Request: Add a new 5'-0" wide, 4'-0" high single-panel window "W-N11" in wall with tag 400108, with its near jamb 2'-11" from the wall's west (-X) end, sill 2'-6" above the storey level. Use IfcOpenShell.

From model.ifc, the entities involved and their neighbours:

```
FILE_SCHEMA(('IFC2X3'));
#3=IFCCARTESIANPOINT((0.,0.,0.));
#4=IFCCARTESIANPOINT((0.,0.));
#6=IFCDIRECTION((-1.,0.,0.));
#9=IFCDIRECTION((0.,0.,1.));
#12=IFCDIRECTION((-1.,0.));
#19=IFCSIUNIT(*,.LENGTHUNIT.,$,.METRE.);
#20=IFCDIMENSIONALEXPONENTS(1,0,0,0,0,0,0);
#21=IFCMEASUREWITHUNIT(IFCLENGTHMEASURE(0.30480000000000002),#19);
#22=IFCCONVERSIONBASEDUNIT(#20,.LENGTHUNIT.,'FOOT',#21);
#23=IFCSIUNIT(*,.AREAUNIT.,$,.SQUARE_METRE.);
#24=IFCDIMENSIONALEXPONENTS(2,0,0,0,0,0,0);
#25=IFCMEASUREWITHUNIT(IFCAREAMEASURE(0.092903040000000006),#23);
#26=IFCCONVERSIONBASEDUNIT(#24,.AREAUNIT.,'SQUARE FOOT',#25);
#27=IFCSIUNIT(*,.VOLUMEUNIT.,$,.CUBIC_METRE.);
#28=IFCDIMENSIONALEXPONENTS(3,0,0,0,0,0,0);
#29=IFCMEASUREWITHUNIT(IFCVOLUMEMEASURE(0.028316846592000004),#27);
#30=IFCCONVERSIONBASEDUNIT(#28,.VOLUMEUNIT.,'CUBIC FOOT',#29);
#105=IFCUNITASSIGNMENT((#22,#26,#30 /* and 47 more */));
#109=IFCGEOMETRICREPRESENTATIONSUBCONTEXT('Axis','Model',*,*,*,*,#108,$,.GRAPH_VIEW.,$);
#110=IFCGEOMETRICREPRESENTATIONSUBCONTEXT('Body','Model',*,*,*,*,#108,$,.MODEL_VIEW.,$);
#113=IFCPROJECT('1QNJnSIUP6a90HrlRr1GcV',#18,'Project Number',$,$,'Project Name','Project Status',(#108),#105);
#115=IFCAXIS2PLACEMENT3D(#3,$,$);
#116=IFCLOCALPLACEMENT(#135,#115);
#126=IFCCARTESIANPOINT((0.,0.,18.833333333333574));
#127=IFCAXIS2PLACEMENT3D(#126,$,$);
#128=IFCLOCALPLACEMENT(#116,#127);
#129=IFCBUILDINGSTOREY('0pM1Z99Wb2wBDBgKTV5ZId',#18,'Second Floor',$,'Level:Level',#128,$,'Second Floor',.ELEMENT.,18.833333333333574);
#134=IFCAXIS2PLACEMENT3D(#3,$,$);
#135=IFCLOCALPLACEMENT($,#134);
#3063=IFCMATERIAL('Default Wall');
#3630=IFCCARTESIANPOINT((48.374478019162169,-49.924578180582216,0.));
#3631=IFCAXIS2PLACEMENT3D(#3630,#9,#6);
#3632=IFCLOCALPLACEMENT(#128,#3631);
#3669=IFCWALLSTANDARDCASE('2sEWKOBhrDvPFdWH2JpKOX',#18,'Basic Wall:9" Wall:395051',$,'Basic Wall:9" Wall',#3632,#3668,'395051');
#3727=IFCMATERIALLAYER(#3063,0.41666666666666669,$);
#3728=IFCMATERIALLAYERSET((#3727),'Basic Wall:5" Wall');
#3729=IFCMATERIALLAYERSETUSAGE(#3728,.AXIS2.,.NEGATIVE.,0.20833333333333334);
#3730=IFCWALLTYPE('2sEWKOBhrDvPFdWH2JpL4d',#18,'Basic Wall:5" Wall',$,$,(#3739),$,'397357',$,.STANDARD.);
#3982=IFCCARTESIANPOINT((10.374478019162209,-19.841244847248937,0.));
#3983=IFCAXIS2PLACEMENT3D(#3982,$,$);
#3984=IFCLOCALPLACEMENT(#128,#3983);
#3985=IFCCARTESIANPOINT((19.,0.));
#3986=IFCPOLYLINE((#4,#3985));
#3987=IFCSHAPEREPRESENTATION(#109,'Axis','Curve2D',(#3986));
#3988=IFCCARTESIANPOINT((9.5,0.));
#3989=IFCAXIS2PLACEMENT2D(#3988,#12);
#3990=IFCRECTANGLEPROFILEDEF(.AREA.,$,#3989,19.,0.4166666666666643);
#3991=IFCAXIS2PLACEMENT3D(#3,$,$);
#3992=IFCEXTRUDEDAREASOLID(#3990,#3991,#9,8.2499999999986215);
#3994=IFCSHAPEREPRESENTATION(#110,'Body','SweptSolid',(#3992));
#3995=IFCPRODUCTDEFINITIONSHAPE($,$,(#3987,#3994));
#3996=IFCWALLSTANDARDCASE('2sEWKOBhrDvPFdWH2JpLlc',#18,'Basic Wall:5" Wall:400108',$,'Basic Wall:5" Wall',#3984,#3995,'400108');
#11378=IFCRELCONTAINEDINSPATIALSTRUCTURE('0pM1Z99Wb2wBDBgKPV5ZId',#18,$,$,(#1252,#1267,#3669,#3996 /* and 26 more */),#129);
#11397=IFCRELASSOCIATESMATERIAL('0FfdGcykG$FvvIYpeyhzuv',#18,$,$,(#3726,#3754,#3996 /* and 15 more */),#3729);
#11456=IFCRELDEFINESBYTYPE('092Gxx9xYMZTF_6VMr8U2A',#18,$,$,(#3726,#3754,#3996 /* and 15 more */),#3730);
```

```python
import numpy as np
import ifcopenshell
import ifcopenshell.api.feature
import ifcopenshell.api.geometry
import ifcopenshell.api.root
import ifcopenshell.api.spatial
import ifcopenshell.api.type
import ifcopenshell.geom
import ifcopenshell.util.element
import ifcopenshell.util.placement
import ifcopenshell.util.representation
import ifcopenshell.util.shape
import ifcopenshell.util.unit

model = ifcopenshell.open("model.ifc")
unit_scale = ifcopenshell.util.unit.calculate_unit_scale(model)
settings = ifcopenshell.geom.settings()


def volume(element):
    """Net volume in cubic metres, openings subtracted."""
    shape = ifcopenshell.geom.create_shape(settings, element)
    return ifcopenshell.util.shape.get_volume(shape.geometry)


wall = model.by_guid("2sEWKOBhrDvPFdWH2JpLlc")
storey = ifcopenshell.util.element.get_container(wall, ifc_class="IfcBuildingStorey")
context = ifcopenshell.util.representation.get_context(model, "Model", "Body", "MODEL_VIEW")
before = volume(wall)

width, height, from_end, sill = 1.524, 1.2192, 0.889, 0.762  # metres

# The wall runs along its own X axis, and the end named is its -X end.
wall_shape = ifcopenshell.geom.create_shape(settings, wall)
x, y, z = ifcopenshell.util.shape.get_vertices(wall_shape.geometry).T
start = x.min() + from_end
face, thickness = float(y.min()), float(y.max() - y.min())
wall_matrix = ifcopenshell.util.placement.get_local_placement(wall.ObjectPlacement)
level = ifcopenshell.util.placement.get_local_placement(storey.ObjectPlacement)[2, 3]


def in_wall(x, y):
    """Placement at x, y metres in the wall's axes, at sill height."""
    matrix = wall_matrix.copy()
    matrix[:, 3] = wall_matrix @ np.array([x / unit_scale, y / unit_scale, 0.0, 1.0])
    matrix[2, 3] = level + sill / unit_scale
    return matrix


# Opening: a box that overshoots both wall faces by 50 mm.
opening = ifcopenshell.api.root.create_entity(model, ifc_class="IfcOpeningElement")
box = ifcopenshell.api.geometry.add_wall_representation(
    model, context=context, length=width, height=height, thickness=thickness + 0.1
)
ifcopenshell.api.geometry.assign_representation(model, product=opening, representation=box)
ifcopenshell.api.geometry.edit_object_placement(model, product=opening, matrix=in_wall(start, face - 0.05), is_si=False)
ifcopenshell.api.feature.add_feature(model, feature=opening, element=wall)

window = ifcopenshell.api.root.create_entity(model, ifc_class="IfcWindow", name="W-N11")
window.OverallWidth, window.OverallHeight = width / unit_scale, height / unit_scale
body = ifcopenshell.api.geometry.add_window_representation(
    model,
    context=context,
    overall_width=window.OverallWidth,
    overall_height=window.OverallHeight,
    partition_type="SINGLE_PANEL",
)
ifcopenshell.api.geometry.assign_representation(model, product=window, representation=body)
ifcopenshell.api.spatial.assign_container(model, products=[window], relating_structure=storey)
fills = ifcopenshell.api.feature.add_filling(model, opening=opening, element=window)
fills.OwnerHistory = window.OwnerHistory  # required in IFC2X3

# IFC2X3 keeps the operation on the window style.
style = ifcopenshell.api.root.create_entity(model, ifc_class="IfcWindowStyle", name="W-N11")
style.OperationType, style.ConstructionType = "SINGLE_PANEL", "NOTDEFINED"
style.ParameterTakesPrecedence = style.Sizeable = False
ifcopenshell.api.type.assign_type(model, related_objects=[window], relating_type=style)

# Centre the window in the wall's thickness.
ifcopenshell.api.geometry.edit_object_placement(model, product=window, matrix=in_wall(start, face), is_si=False)
window_shape = ifcopenshell.geom.create_shape(settings, window)
depth = ifcopenshell.util.shape.get_vertices(window_shape.geometry)[:, 1]
offset = face + thickness / 2 - (depth.min() + depth.max()) / 2
ifcopenshell.api.geometry.edit_object_placement(model, product=window, matrix=in_wall(start, offset), is_si=False)

after = volume(wall)

print(f"wall volume {before:.3f} -> {after:.3f} m3")

model.write("model_edited.ifc")
```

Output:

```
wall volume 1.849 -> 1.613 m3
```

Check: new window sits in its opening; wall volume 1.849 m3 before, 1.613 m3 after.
